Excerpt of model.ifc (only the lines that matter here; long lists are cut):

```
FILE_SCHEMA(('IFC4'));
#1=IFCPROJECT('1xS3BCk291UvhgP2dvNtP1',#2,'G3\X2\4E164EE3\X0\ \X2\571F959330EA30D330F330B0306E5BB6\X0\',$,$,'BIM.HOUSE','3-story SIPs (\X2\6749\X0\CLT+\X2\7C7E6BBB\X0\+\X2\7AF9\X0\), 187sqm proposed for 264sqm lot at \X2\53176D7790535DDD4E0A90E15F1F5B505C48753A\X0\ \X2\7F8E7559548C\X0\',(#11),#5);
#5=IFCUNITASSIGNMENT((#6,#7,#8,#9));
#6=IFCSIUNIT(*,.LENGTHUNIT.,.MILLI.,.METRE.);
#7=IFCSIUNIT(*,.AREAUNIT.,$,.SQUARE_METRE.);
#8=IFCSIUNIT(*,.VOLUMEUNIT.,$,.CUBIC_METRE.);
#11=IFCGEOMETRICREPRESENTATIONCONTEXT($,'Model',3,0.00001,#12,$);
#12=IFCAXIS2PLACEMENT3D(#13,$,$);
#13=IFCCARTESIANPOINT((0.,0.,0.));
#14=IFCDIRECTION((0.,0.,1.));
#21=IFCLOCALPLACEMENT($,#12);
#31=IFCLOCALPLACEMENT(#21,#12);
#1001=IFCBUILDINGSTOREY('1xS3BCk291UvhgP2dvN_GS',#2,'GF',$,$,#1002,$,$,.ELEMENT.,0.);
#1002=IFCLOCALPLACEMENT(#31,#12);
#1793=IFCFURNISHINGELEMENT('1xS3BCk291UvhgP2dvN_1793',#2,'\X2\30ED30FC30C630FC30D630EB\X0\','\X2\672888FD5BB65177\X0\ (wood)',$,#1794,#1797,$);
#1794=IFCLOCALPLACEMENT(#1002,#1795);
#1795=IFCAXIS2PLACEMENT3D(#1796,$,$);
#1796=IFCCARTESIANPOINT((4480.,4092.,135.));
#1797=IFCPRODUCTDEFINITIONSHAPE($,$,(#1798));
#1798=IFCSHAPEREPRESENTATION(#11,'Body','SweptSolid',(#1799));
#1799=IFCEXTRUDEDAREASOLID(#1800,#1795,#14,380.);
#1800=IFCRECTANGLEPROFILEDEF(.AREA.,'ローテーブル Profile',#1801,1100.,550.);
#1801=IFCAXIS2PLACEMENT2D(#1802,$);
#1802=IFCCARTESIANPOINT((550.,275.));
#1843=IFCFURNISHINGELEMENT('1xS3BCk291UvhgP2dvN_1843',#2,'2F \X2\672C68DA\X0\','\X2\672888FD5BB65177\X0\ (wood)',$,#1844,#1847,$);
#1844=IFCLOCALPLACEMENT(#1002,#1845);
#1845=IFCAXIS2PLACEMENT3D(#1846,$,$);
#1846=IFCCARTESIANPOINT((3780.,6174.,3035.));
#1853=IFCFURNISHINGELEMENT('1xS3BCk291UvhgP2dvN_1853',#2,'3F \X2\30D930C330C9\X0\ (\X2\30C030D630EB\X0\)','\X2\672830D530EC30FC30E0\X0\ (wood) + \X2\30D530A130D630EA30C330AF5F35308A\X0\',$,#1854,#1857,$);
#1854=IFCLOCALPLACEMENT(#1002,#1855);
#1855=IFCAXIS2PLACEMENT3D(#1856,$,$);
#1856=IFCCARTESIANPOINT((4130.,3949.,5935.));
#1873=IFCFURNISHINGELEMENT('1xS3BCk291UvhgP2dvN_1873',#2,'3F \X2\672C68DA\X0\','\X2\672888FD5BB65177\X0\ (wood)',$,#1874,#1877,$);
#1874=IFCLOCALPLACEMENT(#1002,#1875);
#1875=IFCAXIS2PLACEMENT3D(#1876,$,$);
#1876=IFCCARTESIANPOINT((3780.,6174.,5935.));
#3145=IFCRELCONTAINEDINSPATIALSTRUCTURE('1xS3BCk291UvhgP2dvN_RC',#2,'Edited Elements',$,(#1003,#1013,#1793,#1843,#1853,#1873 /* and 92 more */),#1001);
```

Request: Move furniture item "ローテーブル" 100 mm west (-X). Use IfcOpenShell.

```python
import ifcopenshell
import ifcopenshell.api.geometry
import ifcopenshell.util.placement
import ifcopenshell.util.unit

model = ifcopenshell.open("model.ifc")
unit_scale = ifcopenshell.util.unit.calculate_unit_scale(model)

item = model.by_id(1793)
matrix = ifcopenshell.util.placement.get_local_placement(item.ObjectPlacement)
matrix[0, 3] -= 0.1 / unit_scale
ifcopenshell.api.geometry.edit_object_placement(model, product=item, matrix=matrix, is_si=False)

print(ifcopenshell.util.placement.get_local_placement(item.ObjectPlacement).round(3) + 0.0)

model.write("model_edited.ifc")
```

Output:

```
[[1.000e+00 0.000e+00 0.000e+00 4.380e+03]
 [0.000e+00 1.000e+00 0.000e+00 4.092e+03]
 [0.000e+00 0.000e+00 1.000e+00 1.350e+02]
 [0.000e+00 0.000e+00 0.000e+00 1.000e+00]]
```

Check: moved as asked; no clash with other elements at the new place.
